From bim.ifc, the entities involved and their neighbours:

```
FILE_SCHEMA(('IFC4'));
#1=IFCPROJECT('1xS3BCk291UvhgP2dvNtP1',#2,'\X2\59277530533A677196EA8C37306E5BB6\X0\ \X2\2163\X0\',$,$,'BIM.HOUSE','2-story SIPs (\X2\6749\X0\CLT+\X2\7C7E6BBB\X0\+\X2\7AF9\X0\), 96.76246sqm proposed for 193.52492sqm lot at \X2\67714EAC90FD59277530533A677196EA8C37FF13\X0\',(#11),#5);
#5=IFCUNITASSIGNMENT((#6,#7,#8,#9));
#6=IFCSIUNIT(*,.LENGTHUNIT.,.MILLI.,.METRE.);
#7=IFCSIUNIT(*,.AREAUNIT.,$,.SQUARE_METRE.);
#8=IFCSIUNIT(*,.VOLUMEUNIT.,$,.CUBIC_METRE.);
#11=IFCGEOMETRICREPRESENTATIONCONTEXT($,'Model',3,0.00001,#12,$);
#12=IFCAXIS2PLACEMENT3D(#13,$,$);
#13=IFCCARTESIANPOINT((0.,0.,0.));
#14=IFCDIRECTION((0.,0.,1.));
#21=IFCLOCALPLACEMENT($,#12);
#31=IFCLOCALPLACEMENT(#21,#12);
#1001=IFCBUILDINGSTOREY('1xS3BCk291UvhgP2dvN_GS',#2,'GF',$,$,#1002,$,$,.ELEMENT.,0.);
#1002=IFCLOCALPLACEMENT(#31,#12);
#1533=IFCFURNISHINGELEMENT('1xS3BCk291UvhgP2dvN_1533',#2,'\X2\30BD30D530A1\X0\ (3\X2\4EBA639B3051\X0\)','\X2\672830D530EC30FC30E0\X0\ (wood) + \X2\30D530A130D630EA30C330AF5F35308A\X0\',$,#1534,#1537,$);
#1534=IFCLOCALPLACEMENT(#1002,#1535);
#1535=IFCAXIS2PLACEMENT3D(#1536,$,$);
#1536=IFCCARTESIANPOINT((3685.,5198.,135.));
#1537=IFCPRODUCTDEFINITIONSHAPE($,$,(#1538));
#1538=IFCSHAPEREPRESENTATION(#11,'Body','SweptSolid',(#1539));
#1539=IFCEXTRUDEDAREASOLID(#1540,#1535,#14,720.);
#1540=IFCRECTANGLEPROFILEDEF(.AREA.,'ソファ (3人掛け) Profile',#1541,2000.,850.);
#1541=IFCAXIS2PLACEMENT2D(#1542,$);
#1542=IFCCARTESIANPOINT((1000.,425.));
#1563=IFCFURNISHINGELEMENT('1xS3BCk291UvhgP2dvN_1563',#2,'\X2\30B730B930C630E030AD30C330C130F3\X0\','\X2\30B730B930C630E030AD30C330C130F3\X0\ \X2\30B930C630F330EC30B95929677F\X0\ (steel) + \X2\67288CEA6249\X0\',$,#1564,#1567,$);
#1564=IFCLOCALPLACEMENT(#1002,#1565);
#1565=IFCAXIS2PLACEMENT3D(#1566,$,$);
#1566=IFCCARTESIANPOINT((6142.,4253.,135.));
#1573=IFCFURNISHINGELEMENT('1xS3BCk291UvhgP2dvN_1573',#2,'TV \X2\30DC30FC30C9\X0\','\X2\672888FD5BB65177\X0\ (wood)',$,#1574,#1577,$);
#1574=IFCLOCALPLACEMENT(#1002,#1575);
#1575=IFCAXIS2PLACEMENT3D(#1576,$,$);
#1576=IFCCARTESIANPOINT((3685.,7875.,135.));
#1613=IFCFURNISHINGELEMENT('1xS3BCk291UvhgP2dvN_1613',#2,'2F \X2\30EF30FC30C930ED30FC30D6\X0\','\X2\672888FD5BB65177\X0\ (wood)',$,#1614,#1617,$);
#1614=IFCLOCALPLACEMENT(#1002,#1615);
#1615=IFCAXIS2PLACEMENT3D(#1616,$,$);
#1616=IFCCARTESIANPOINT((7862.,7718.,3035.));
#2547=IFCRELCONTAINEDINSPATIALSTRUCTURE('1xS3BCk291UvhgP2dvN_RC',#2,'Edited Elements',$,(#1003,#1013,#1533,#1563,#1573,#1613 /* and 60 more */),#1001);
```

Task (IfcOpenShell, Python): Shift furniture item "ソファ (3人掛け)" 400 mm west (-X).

```python
import ifcopenshell
import ifcopenshell.api.geometry
import ifcopenshell.util.placement

model = ifcopenshell.open("bim.ifc")

item = model.by_guid("1xS3BCk291UvhgP2dvN_1533")
matrix = ifcopenshell.util.placement.get_local_placement(item.ObjectPlacement)
matrix[0, 3] -= 400.0
ifcopenshell.api.geometry.edit_object_placement(model, product=item, matrix=matrix, is_si=False)

print(ifcopenshell.util.placement.get_local_placement(item.ObjectPlacement).round(3) + 0.0)

model.write("bim_rev.ifc")
```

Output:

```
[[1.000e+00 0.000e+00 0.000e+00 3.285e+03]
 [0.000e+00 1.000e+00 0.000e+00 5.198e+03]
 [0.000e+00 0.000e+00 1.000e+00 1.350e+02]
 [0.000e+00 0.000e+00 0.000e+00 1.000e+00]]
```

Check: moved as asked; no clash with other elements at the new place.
